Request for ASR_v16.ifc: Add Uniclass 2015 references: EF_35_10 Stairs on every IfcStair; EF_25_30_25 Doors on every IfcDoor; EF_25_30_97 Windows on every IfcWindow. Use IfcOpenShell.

First a look at what the model holds.

```python
import ifcopenshell

model = ifcopenshell.open("ASR_v16.ifc")
print(model.schema)
print("classifications:", [c.Name for c in model.by_type("IfcClassification")])
for ifc_class in ("IfcDoor", "IfcRoof", "IfcStair", "IfcWall", "IfcWindow"):
    print(ifc_class, len(model.by_type(ifc_class)))
```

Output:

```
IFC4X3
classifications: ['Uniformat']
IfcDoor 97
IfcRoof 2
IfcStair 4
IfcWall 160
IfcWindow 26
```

```python
import ifcopenshell
import ifcopenshell.api.classification

model = ifcopenshell.open("ASR_v16.ifc")

system = ifcopenshell.api.classification.add_classification(model, classification="Uniclass 2015")

codes = {
    "IfcStair": ("EF_35_10", "Stairs"),
    "IfcDoor": ("EF_25_30_25", "Doors"),
    "IfcWindow": ("EF_25_30_97", "Windows"),
}
for ifc_class, (code, name) in codes.items():
    products = model.by_type(ifc_class)
    ifcopenshell.api.classification.add_reference(
        model, products=products, classification=system, identification=code, name=name
    )
    print(code, len(products))

model.write("ASR_v16-out.ifc")
```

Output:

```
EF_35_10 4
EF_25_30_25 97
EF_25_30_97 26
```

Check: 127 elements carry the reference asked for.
